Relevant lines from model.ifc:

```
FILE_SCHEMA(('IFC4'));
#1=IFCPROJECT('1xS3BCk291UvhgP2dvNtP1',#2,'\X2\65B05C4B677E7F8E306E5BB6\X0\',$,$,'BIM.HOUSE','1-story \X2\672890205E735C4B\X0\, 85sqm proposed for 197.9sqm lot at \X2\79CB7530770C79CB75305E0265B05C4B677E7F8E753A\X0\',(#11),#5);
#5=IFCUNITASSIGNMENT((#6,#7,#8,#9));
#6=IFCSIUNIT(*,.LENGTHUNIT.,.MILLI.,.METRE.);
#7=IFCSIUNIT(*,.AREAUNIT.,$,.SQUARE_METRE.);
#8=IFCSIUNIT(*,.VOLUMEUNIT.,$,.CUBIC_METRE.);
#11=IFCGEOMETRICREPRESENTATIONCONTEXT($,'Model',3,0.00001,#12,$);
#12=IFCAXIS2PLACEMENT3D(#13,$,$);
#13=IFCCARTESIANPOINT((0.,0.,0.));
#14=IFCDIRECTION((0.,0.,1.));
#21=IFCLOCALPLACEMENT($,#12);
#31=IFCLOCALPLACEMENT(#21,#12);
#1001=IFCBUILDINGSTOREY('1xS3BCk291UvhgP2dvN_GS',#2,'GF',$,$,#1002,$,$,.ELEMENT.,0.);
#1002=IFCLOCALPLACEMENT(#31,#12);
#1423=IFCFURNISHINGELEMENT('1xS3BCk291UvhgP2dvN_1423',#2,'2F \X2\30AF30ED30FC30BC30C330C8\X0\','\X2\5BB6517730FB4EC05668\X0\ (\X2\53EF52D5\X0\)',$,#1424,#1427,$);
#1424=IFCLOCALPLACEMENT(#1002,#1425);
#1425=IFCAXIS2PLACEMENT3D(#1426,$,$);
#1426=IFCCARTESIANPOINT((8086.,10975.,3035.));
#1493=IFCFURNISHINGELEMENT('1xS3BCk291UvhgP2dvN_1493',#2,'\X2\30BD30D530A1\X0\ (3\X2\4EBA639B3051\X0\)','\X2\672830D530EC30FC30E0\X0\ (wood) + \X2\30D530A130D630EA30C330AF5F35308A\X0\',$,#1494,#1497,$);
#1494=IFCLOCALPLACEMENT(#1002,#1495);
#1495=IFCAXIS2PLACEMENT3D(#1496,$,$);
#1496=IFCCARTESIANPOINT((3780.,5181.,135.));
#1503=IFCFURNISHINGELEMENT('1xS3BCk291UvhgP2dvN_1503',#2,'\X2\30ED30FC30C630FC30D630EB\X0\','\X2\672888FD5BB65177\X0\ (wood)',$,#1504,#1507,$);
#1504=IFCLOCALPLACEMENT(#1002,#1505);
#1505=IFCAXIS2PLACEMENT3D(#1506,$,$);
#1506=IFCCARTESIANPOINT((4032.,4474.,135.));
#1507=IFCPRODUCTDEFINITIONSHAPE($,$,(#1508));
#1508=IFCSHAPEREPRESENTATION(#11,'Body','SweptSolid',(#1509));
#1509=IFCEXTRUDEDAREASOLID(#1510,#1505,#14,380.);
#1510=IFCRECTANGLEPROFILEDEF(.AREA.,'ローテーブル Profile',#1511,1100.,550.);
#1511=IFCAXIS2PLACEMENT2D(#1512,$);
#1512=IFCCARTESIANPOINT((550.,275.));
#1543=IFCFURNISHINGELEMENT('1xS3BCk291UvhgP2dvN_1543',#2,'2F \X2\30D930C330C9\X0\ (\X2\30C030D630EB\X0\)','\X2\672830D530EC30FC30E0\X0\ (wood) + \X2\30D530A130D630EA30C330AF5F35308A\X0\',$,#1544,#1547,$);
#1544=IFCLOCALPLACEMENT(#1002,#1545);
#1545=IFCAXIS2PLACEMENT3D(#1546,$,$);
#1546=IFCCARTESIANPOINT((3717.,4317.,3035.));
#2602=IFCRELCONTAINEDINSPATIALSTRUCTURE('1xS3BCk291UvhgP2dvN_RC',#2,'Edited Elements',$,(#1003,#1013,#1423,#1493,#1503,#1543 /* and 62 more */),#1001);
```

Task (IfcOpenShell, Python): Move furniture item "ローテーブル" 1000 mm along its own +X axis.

```python
import ifcopenshell
import ifcopenshell.api.geometry
import ifcopenshell.util.placement

model = ifcopenshell.open("model.ifc")

item = model.by_guid("1xS3BCk291UvhgP2dvN_1503")
matrix = ifcopenshell.util.placement.get_local_placement(item.ObjectPlacement)
matrix[:3, 3] += matrix[:3, 0] * 1000.0
ifcopenshell.api.geometry.edit_object_placement(model, product=item, matrix=matrix, is_si=False)

print(ifcopenshell.util.placement.get_local_placement(item.ObjectPlacement).round(3) + 0.0)

model.write("model_rev.ifc")
```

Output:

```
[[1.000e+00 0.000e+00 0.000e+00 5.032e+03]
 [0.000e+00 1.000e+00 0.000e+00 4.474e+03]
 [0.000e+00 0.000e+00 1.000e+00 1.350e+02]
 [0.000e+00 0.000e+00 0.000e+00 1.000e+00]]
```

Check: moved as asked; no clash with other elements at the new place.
